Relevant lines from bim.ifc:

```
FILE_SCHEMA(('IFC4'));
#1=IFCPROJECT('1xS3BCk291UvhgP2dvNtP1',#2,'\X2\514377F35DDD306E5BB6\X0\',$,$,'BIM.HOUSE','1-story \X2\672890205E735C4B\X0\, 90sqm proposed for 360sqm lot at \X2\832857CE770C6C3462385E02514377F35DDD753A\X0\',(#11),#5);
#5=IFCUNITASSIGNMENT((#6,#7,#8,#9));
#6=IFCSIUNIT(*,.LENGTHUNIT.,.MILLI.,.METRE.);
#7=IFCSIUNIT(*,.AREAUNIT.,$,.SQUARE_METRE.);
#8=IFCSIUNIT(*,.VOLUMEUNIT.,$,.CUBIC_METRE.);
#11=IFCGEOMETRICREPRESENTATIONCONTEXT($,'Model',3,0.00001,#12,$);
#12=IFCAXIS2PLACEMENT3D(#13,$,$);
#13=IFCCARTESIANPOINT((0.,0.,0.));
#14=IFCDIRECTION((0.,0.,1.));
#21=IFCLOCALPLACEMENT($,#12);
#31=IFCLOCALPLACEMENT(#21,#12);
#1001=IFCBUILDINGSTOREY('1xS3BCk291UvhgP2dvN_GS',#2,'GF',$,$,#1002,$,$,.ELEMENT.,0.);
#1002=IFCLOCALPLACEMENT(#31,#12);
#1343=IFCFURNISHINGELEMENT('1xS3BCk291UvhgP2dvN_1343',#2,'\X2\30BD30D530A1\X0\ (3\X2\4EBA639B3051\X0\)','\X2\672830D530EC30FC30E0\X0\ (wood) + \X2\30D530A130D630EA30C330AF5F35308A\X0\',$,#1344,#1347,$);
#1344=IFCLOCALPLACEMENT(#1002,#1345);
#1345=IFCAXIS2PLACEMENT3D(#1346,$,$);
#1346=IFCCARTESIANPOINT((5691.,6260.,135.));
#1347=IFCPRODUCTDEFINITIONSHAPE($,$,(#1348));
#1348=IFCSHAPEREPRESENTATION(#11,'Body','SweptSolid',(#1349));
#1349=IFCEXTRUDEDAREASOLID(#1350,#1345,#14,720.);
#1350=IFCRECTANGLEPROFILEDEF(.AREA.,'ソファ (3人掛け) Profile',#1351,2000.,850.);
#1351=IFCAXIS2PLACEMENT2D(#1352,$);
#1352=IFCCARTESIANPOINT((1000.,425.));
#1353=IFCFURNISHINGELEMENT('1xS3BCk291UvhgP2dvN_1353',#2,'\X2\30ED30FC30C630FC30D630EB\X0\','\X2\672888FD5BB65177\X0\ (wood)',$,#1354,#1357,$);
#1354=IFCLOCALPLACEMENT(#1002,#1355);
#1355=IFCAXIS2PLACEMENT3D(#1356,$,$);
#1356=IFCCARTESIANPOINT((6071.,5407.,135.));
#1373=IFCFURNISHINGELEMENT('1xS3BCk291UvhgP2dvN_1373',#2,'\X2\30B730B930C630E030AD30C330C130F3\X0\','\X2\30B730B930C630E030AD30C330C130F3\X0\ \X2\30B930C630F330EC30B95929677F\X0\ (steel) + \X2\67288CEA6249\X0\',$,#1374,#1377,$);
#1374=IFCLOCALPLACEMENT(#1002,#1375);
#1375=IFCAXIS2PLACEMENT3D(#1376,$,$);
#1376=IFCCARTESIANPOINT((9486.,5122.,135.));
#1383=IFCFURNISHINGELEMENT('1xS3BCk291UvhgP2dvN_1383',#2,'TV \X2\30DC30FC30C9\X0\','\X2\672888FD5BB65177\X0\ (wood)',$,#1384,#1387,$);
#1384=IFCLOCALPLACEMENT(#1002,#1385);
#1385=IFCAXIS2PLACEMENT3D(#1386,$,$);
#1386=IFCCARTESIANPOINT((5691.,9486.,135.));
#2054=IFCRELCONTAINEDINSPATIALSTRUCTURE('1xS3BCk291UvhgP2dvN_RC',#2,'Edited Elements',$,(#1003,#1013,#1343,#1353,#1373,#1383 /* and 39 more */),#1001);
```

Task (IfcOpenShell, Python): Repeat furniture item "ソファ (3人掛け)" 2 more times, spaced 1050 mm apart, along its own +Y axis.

```python
import ifcopenshell
import ifcopenshell.api.geometry
import ifcopenshell.api.root
import ifcopenshell.util.element
import ifcopenshell.util.placement

model = ifcopenshell.open("bim.ifc")


def reuse_history(source, copy):
    """copy_class also copies each property set's owner history, people and application; keep the originals."""
    for rel in copy.IsDefinedBy:
        if rel.is_a("IfcRelDefinesByProperties") and (history := rel.RelatingPropertyDefinition.OwnerHistory):
            rel.RelatingPropertyDefinition.OwnerHistory = source.OwnerHistory
            ifcopenshell.util.element.remove_deep2(model, history)


source = model.by_guid("1xS3BCk291UvhgP2dvN_1343")
base = ifcopenshell.util.placement.get_local_placement(source.ObjectPlacement)
step = base[:3, 1] * 1050.0

for i in range(1, 3):
    copy = ifcopenshell.api.root.copy_class(model, product=source)
    copy.Representation = ifcopenshell.util.element.copy_deep(
        model, source.Representation, exclude=["IfcGeometricRepresentationContext", "IfcRepresentationMap"]
    )
    reuse_history(source, copy)
    matrix = base.copy()
    matrix[:3, 3] += i * step
    print("added at", matrix[:3, 3].round(3) + 0.0)
    ifcopenshell.api.geometry.edit_object_placement(model, product=copy, matrix=matrix, is_si=False)

model.write("bim_updated.ifc")
```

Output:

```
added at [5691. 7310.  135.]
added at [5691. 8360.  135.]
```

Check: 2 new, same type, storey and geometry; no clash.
